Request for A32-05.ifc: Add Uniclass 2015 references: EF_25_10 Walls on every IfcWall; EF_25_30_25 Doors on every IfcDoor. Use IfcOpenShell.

First a look at what the model holds.

```python
import ifcopenshell

model = ifcopenshell.open("A32-05.ifc")
print(model.schema)
print("classifications:", [c.Name for c in model.by_type("IfcClassification")])
for ifc_class in ("IfcDoor", "IfcRoof", "IfcStair", "IfcWall", "IfcWindow"):
    print(ifc_class, len(model.by_type(ifc_class)))
```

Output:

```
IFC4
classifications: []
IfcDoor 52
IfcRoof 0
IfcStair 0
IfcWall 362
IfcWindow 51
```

```python
import ifcopenshell
import ifcopenshell.api.classification

model = ifcopenshell.open("A32-05.ifc")

system = ifcopenshell.api.classification.add_classification(model, classification="Uniclass 2015")

codes = {
    "IfcWall": ("EF_25_10", "Walls"),
    "IfcDoor": ("EF_25_30_25", "Doors"),
}
for ifc_class, (code, name) in codes.items():
    products = model.by_type(ifc_class)
    ifcopenshell.api.classification.add_reference(
        model, products=products, classification=system, identification=code, name=name
    )
    print(code, len(products))

model.write("A32-05-out.ifc")
```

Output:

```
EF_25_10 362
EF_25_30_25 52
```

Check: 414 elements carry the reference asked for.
